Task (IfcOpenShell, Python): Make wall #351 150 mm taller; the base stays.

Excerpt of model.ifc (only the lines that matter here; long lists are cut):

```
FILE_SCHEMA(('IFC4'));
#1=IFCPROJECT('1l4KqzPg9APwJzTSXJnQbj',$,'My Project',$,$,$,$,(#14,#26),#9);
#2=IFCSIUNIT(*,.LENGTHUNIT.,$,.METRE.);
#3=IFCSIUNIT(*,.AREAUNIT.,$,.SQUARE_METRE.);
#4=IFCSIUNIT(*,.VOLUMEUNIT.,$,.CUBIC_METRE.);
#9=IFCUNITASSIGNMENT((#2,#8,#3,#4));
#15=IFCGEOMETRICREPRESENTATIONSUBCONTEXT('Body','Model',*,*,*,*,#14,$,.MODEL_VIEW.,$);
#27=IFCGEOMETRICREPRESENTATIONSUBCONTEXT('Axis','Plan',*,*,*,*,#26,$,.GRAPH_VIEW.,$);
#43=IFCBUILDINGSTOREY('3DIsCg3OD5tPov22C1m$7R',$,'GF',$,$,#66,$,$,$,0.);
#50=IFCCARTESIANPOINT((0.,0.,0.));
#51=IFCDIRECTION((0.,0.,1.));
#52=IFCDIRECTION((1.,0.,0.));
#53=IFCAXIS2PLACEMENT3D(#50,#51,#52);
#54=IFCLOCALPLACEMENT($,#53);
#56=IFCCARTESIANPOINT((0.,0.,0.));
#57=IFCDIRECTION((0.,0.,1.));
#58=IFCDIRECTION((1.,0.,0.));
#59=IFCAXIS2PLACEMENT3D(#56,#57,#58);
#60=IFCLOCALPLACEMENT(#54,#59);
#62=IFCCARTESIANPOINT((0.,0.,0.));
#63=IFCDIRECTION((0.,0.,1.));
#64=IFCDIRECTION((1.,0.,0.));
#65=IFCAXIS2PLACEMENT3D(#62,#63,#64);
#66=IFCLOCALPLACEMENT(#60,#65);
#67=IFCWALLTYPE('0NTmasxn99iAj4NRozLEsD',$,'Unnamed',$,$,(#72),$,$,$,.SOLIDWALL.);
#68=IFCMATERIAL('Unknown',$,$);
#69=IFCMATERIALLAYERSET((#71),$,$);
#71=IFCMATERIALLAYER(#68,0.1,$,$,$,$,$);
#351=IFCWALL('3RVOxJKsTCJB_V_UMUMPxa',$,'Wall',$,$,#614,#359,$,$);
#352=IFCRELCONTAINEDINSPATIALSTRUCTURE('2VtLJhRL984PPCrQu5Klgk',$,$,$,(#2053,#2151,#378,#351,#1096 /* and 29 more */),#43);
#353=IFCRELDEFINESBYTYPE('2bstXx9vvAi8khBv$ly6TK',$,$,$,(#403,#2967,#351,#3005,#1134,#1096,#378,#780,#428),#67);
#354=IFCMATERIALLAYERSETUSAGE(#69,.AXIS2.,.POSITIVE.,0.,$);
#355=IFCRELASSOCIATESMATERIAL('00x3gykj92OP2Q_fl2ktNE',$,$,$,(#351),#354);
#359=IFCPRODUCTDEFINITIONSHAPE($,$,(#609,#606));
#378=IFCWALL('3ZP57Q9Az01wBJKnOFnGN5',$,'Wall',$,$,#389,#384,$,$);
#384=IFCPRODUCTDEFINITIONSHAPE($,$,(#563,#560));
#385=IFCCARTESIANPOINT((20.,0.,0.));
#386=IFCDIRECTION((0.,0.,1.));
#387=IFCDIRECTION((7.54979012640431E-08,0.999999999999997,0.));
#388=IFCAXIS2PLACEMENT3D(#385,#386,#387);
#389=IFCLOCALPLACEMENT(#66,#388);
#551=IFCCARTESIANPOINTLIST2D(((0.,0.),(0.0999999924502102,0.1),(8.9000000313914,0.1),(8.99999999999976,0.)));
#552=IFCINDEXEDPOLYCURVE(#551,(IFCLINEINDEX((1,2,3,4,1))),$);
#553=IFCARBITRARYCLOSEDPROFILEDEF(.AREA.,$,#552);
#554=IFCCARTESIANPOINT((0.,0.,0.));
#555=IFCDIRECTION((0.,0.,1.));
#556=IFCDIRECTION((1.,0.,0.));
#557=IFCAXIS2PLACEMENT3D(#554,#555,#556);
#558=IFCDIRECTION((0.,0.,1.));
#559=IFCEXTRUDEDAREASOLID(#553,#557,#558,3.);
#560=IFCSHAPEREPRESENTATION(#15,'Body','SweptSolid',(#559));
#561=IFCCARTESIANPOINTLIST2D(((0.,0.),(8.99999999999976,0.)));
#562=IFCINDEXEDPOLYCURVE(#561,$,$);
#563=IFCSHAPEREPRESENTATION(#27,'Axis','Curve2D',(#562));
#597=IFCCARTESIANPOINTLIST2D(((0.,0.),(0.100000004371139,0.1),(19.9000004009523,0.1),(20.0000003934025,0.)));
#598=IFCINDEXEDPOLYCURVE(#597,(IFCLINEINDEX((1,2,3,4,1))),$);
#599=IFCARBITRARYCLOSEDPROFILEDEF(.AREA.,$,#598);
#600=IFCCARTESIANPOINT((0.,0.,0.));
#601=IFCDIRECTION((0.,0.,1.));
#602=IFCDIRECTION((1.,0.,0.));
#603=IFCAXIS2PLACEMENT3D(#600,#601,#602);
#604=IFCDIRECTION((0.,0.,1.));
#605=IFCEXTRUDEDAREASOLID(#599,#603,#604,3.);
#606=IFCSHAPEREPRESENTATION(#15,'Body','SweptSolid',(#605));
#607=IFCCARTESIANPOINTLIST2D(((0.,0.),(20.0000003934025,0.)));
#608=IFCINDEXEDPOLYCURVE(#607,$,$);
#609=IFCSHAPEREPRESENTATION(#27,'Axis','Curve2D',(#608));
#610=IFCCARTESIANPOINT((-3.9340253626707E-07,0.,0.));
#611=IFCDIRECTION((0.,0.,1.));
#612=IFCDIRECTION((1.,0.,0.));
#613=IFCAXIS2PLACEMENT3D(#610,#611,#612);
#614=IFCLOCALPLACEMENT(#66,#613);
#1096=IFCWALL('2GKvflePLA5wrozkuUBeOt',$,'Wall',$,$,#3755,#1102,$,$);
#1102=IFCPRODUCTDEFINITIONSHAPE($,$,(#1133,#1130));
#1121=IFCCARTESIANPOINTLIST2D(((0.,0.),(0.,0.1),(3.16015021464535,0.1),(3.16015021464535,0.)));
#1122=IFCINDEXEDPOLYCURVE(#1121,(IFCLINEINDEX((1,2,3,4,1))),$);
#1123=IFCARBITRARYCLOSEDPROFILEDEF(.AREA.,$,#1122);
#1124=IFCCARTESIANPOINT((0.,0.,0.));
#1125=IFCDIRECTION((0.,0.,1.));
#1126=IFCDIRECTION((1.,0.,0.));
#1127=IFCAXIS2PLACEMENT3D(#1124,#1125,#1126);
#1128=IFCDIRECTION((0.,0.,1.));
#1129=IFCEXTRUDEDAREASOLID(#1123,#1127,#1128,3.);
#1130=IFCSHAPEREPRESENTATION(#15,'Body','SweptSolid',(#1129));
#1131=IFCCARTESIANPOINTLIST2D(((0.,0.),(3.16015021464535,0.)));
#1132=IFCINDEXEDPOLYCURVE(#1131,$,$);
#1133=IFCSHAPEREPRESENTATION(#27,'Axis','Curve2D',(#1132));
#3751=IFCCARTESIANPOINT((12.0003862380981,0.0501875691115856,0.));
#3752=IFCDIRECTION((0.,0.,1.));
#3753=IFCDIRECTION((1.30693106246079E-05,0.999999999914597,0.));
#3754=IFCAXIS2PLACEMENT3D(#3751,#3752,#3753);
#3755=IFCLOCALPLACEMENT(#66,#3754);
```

```python
import ifcopenshell
import ifcopenshell.geom
import ifcopenshell.util.representation
import ifcopenshell.util.shape
import ifcopenshell.util.unit

model = ifcopenshell.open("model.ifc")
unit_scale = ifcopenshell.util.unit.calculate_unit_scale(model)
settings = ifcopenshell.geom.settings()


def volume(element):
    """Net volume in cubic metres, openings subtracted."""
    shape = ifcopenshell.geom.create_shape(settings, element)
    return ifcopenshell.util.shape.get_volume(shape.geometry)


wall = model.by_guid("3RVOxJKsTCJB_V_UMUMPxa")
before = volume(wall)

body = ifcopenshell.util.representation.get_representation(wall, "Model", "Body")
solid = body.Items[0]
old_height = solid.Depth
solid.Depth += 0.15 / unit_scale
after = volume(wall)

print(f"height {old_height:g} -> {solid.Depth:g}, volume {before:.3f} -> {after:.3f} m3")

model.write("model-out.ifc")
```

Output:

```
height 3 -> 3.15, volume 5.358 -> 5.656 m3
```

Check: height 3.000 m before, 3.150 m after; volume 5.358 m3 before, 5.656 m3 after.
